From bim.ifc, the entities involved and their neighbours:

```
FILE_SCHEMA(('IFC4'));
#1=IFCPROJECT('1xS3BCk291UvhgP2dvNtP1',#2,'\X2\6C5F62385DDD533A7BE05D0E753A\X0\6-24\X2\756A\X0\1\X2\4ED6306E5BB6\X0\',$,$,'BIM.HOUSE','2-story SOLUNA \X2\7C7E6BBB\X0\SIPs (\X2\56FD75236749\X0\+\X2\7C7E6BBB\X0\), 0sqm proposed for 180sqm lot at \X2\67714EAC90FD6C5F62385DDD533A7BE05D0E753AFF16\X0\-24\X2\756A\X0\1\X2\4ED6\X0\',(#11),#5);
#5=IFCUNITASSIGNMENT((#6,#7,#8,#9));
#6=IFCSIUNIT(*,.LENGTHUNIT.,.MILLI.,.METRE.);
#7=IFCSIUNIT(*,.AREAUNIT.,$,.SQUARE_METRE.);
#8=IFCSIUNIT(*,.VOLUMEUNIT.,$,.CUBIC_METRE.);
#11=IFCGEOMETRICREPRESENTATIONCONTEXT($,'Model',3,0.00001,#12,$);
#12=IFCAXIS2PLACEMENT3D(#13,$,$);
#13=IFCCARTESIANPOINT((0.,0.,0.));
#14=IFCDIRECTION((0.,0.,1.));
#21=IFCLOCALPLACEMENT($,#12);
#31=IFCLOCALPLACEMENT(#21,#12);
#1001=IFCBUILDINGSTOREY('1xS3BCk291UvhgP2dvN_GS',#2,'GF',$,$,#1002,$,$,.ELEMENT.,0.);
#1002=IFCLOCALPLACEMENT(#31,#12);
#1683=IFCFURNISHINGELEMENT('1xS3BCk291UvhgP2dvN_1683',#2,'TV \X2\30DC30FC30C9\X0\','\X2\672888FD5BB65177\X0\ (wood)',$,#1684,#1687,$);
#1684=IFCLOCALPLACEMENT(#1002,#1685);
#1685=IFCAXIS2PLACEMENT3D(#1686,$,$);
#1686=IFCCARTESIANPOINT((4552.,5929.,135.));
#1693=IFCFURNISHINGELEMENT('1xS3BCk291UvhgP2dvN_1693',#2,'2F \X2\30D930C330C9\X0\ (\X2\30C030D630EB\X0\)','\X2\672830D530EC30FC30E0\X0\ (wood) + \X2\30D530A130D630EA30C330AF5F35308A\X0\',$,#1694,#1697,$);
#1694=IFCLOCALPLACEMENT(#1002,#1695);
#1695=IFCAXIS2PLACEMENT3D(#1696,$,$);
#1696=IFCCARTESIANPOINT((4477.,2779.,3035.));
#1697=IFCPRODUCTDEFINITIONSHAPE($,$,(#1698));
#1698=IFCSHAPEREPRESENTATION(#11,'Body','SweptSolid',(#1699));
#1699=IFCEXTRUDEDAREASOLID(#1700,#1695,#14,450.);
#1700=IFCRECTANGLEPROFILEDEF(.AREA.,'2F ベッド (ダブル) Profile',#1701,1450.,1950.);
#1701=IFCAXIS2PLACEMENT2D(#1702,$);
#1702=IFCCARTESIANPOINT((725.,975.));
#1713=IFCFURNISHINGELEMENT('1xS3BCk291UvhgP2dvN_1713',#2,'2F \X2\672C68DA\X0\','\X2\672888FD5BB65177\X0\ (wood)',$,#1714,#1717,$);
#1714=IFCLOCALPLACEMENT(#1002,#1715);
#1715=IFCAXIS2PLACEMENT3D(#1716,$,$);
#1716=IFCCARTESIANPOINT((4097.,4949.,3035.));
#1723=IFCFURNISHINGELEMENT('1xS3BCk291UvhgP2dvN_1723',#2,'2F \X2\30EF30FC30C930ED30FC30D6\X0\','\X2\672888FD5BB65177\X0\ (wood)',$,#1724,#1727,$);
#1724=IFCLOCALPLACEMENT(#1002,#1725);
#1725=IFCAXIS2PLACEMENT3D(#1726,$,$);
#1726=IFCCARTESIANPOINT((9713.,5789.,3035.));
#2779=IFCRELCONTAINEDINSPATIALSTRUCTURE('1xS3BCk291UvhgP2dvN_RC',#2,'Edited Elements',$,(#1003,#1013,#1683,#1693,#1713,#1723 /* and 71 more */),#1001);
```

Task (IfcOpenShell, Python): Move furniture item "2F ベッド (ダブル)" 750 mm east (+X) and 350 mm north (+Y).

```python
import ifcopenshell
import ifcopenshell.api.geometry
import ifcopenshell.util.placement
import ifcopenshell.util.unit

model = ifcopenshell.open("bim.ifc")
unit_scale = ifcopenshell.util.unit.calculate_unit_scale(model)

item = model.by_id(1693)
matrix = ifcopenshell.util.placement.get_local_placement(item.ObjectPlacement)
matrix[0, 3] += 0.75 / unit_scale
matrix[1, 3] += 0.35 / unit_scale
ifcopenshell.api.geometry.edit_object_placement(model, product=item, matrix=matrix, is_si=False)

print(ifcopenshell.util.placement.get_local_placement(item.ObjectPlacement).round(3) + 0.0)

model.write("bim-out.ifc")
```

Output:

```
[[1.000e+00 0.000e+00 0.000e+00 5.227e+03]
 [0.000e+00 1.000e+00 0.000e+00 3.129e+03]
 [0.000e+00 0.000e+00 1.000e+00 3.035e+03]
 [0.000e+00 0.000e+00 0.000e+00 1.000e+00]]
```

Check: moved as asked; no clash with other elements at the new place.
